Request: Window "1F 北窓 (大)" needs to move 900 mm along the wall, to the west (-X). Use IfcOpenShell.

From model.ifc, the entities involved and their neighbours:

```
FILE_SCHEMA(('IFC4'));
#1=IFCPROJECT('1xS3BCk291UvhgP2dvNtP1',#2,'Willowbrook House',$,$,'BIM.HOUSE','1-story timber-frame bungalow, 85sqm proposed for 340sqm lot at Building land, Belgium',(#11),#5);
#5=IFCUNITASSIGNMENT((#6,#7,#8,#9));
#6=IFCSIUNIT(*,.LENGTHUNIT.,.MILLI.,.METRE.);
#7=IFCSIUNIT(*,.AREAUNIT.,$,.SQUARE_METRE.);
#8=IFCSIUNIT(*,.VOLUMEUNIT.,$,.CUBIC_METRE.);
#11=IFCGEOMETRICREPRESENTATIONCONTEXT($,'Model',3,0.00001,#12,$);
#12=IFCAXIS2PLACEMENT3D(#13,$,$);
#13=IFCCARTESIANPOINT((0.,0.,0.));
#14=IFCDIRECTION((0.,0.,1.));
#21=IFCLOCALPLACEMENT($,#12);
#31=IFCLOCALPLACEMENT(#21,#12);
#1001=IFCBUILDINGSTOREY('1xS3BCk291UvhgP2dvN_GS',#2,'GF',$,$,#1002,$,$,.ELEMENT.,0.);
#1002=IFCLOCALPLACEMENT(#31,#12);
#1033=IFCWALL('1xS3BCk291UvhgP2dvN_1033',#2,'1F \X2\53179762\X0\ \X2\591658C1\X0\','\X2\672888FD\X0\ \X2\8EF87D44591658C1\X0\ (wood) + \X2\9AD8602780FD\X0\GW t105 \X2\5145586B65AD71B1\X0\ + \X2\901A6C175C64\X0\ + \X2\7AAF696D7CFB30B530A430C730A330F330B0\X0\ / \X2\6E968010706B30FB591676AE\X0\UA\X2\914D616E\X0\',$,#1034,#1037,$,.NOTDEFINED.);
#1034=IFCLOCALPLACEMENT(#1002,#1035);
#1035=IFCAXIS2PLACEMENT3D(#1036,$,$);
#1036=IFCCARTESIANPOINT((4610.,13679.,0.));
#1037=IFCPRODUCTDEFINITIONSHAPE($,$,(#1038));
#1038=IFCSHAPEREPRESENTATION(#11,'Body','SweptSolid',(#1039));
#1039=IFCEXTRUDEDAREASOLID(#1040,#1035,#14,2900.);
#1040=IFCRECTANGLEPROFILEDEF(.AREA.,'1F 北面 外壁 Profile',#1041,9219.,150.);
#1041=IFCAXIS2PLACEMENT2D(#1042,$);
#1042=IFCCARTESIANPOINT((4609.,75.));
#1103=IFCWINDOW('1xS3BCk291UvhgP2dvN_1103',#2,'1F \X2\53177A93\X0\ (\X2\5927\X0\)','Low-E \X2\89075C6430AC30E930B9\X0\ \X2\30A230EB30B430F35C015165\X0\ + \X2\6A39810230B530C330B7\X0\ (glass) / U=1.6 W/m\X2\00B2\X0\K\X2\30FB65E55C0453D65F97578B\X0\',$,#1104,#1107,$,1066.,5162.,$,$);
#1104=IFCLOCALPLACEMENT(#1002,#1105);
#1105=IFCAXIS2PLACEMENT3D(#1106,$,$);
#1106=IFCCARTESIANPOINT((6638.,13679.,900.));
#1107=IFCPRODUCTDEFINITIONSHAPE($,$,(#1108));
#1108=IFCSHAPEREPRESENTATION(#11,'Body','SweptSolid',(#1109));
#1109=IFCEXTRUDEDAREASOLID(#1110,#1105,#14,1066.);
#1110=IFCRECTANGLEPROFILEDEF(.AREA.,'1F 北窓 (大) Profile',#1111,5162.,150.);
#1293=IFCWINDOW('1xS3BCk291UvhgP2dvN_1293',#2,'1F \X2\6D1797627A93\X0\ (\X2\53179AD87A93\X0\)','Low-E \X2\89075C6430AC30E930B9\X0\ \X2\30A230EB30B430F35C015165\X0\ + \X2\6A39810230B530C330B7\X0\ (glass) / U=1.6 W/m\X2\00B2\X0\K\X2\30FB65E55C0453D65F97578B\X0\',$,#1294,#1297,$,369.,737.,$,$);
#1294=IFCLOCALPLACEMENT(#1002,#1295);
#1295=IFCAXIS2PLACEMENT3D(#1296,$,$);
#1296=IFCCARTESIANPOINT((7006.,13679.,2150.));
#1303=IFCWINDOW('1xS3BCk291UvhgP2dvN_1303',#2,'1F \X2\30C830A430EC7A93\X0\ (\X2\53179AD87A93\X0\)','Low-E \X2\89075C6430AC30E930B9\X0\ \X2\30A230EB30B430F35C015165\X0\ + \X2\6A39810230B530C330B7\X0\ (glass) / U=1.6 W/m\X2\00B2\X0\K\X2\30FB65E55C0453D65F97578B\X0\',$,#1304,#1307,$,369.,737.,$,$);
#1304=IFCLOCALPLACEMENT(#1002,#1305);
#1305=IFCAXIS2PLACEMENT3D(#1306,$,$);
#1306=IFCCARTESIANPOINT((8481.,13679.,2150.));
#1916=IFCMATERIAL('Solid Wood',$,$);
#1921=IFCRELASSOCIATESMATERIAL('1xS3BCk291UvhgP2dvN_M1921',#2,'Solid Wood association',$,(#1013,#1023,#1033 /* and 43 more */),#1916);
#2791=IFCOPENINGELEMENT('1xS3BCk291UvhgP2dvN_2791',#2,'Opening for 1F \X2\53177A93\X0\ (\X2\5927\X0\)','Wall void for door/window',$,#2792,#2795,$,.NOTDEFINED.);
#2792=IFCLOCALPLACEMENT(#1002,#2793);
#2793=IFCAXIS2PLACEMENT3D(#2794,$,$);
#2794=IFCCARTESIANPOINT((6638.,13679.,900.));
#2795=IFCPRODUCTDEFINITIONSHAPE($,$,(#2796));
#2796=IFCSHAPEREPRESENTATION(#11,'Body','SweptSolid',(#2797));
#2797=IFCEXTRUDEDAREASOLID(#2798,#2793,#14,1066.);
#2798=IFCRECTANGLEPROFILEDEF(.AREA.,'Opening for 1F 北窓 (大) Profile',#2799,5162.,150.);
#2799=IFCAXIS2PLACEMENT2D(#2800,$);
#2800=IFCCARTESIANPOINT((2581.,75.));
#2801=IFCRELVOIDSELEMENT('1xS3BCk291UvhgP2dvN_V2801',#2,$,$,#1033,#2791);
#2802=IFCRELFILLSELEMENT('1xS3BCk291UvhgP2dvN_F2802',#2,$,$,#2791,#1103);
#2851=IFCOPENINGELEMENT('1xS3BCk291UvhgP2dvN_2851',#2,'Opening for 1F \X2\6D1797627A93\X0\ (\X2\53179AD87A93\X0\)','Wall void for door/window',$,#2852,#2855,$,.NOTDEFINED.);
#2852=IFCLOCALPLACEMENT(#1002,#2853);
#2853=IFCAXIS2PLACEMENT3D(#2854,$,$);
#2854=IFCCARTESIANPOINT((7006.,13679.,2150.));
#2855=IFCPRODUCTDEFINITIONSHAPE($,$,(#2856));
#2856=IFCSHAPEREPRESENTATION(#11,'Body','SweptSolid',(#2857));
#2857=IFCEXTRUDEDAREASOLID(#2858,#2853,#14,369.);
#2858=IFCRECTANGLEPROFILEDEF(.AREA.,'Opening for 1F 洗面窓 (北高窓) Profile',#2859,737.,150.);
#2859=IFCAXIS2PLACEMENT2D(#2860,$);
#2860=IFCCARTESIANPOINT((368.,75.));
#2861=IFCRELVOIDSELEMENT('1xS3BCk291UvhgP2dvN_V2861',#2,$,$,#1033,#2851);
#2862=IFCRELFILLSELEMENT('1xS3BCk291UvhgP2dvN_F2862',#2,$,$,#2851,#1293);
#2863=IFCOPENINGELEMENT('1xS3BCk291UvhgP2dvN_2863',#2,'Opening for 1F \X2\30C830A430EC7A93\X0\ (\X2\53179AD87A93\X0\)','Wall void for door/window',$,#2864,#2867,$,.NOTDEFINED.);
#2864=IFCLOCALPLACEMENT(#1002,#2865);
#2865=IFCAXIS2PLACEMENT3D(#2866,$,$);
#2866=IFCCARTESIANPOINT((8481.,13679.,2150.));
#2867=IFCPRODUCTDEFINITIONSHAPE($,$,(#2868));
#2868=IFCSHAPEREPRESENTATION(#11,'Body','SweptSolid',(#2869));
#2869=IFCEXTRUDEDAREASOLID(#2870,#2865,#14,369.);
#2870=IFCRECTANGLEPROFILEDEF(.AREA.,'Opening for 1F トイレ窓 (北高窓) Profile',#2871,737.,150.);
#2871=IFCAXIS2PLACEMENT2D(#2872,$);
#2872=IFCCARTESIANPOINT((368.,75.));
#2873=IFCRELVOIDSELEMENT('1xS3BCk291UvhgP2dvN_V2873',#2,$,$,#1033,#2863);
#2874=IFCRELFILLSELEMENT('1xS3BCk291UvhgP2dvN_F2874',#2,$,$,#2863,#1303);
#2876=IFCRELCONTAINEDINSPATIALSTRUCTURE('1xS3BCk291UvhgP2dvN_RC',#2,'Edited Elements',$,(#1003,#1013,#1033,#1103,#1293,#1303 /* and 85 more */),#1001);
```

```python
import ifcopenshell
import ifcopenshell.api.geometry
import ifcopenshell.util.placement
import ifcopenshell.util.unit

model = ifcopenshell.open("model.ifc")
unit_scale = ifcopenshell.util.unit.calculate_unit_scale(model)

window = model.by_id(1103)
opening = window.FillsVoids[0].RelatingOpeningElement
wall = opening.VoidsElements[0].RelatingBuildingElement

wall_matrix = ifcopenshell.util.placement.get_local_placement(wall.ObjectPlacement)
shift = wall_matrix[:3, 0] * -0.9 / unit_scale
before = ifcopenshell.util.placement.get_local_placement(window.ObjectPlacement)[:3, 3].copy()

# The window is not placed relative to its opening, so move both.
for product in (opening, window):
    matrix = ifcopenshell.util.placement.get_local_placement(product.ObjectPlacement)
    matrix[:3, 3] += shift
    ifcopenshell.api.geometry.edit_object_placement(model, product=product, matrix=matrix, is_si=False)

after = ifcopenshell.util.placement.get_local_placement(window.ObjectPlacement)[:3, 3]
print("window moved by", (after - before).round(3) + 0.0)

model.write("model_rev.ifc")
```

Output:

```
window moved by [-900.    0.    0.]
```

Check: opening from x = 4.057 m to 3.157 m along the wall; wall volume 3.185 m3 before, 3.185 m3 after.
